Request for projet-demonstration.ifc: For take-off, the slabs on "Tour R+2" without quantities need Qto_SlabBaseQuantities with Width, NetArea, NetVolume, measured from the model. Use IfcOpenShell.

First a look at what the model holds.

```python
import ifcopenshell
import ifcopenshell.util.element
import ifcopenshell.util.unit

model = ifcopenshell.open("projet-demonstration.ifc")
print(model.schema)
for unit_type in ("LENGTHUNIT", "AREAUNIT", "VOLUMEUNIT"):
    print(unit_type, ifcopenshell.util.unit.calculate_unit_scale(model, unit_type))
storey = next(s for s in model.by_type("IfcBuildingStorey") if s.Name == "Tour R+2")
slabs = [e for e in ifcopenshell.util.element.get_decomposition(storey) if e.is_a("IfcSlab")]
for e in sorted(slabs, key=lambda e: e.id()):
    print(e.id(), e.is_a(), e.Name, list(ifcopenshell.util.element.get_psets(e, qtos_only=True)), sep=" | ")
```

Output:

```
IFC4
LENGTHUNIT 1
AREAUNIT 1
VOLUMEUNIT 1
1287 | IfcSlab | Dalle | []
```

```python
import ifcopenshell
import ifcopenshell.api.pset
import ifcopenshell.geom
import ifcopenshell.util.element
import ifcopenshell.util.shape
import ifcopenshell.util.unit

model = ifcopenshell.open("projet-demonstration.ifc")
unit_scale = ifcopenshell.util.unit.calculate_unit_scale(model)
area_scale = ifcopenshell.util.unit.calculate_unit_scale(model, "AREAUNIT")
volume_scale = ifcopenshell.util.unit.calculate_unit_scale(model, "VOLUMEUNIT")
settings = ifcopenshell.geom.settings()

storey = next(s for s in model.by_type("IfcBuildingStorey") if s.Name == "Tour R+2")
slabs = [e for e in ifcopenshell.util.element.get_decomposition(storey) if e.is_a("IfcSlab")]

for e in sorted(slabs, key=lambda e: e.id()):
    if ifcopenshell.util.element.get_psets(e, qtos_only=True, should_inherit=False):
        continue
    # Geometry comes back in metres, in the element's own axes.
    shape = ifcopenshell.geom.create_shape(settings, e)
    values = {
        "Width": ifcopenshell.util.shape.get_z(shape.geometry) / unit_scale,
        "NetArea": ifcopenshell.util.shape.get_footprint_area(shape.geometry) / area_scale,
        "NetVolume": ifcopenshell.util.shape.get_volume(shape.geometry) / volume_scale,
    }
    qto = ifcopenshell.api.pset.add_qto(model, product=e, name="Qto_SlabBaseQuantities")
    ifcopenshell.api.pset.edit_qto(model, qto=qto, properties=values)
    print(e.id(), {k: round(v, 3) for k, v in values.items()})

model.write("projet-demonstration_updated.ifc")
```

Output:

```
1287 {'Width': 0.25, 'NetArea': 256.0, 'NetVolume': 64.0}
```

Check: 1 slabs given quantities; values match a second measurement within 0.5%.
